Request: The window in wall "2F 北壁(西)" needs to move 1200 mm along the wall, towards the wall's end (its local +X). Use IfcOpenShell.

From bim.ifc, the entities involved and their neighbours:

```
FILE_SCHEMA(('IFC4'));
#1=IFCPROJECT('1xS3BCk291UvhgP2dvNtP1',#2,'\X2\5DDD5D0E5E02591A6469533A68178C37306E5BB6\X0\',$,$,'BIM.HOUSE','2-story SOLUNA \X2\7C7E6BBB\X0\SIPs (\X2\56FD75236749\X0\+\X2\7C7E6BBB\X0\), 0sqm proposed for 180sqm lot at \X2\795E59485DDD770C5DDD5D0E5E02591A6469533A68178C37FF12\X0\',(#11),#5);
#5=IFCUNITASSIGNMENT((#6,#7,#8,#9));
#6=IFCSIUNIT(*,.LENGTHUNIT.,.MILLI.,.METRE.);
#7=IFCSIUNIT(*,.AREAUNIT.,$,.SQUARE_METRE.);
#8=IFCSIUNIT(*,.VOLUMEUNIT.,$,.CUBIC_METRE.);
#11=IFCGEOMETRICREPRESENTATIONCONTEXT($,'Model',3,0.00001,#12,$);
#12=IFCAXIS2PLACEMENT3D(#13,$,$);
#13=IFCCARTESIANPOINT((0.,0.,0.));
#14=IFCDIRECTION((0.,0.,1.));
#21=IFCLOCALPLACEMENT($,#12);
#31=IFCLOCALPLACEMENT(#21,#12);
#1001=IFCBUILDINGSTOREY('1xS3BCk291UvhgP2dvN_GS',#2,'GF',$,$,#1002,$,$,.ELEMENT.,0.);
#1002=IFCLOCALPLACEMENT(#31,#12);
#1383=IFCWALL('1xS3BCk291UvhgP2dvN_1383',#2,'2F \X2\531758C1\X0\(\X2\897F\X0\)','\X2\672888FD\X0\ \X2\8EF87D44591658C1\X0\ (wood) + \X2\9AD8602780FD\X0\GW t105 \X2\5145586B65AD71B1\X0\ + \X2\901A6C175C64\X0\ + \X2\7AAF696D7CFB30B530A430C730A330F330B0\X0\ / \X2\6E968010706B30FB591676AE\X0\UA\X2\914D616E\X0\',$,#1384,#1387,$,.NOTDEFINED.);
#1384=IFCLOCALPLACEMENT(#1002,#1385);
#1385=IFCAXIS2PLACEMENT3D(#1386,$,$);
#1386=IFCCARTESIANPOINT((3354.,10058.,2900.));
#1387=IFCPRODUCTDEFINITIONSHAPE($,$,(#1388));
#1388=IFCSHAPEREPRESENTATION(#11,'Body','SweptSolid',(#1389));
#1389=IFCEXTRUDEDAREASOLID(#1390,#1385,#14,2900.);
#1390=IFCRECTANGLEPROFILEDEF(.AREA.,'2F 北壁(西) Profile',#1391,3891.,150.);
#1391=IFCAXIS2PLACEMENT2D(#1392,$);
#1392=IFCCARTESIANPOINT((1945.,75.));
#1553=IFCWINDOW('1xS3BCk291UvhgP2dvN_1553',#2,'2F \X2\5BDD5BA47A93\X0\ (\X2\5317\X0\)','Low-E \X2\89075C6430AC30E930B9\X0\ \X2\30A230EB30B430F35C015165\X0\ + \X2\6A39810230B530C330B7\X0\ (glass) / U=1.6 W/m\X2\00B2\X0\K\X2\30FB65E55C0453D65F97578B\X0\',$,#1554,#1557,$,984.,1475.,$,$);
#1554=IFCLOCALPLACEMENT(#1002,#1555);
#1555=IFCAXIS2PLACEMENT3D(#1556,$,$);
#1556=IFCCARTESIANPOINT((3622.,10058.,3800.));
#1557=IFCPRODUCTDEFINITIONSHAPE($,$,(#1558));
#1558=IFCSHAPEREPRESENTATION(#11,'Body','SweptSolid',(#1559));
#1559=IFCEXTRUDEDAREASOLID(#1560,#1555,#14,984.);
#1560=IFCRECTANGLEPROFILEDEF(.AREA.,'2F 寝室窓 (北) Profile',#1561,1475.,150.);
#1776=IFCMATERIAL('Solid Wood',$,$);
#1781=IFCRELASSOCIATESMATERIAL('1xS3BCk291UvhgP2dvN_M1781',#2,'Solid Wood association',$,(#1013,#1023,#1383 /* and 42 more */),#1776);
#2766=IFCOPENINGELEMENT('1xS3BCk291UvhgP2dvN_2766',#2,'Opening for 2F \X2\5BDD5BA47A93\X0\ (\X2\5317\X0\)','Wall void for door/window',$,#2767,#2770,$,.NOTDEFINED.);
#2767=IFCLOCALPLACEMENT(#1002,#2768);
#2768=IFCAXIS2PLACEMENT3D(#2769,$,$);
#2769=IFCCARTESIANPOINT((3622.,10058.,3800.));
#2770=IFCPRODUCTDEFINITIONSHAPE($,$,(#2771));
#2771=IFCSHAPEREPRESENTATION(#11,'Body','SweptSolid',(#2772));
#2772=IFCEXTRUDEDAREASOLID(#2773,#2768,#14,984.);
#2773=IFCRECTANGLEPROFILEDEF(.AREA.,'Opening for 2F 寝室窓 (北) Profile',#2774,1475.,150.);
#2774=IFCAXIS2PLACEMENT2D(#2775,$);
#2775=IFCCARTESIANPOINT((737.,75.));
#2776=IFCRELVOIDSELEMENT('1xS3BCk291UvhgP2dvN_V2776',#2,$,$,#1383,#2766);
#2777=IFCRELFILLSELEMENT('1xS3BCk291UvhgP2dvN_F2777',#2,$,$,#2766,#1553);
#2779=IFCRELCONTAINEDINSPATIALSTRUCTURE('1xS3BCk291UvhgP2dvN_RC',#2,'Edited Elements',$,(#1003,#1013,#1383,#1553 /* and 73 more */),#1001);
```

```python
import ifcopenshell
import ifcopenshell.api.geometry
import ifcopenshell.util.placement
import ifcopenshell.util.unit

model = ifcopenshell.open("bim.ifc")
unit_scale = ifcopenshell.util.unit.calculate_unit_scale(model)

window = model.by_guid("1xS3BCk291UvhgP2dvN_1553")
opening = window.FillsVoids[0].RelatingOpeningElement
wall = opening.VoidsElements[0].RelatingBuildingElement

wall_matrix = ifcopenshell.util.placement.get_local_placement(wall.ObjectPlacement)
shift = wall_matrix[:3, 0] * 1.2 / unit_scale
before = ifcopenshell.util.placement.get_local_placement(window.ObjectPlacement)[:3, 3].copy()

# The window is not placed relative to its opening, so move both.
for product in (opening, window):
    matrix = ifcopenshell.util.placement.get_local_placement(product.ObjectPlacement)
    matrix[:3, 3] += shift
    ifcopenshell.api.geometry.edit_object_placement(model, product=product, matrix=matrix, is_si=False)

after = ifcopenshell.util.placement.get_local_placement(window.ObjectPlacement)[:3, 3]
print("window moved by", (after - before).round(3) + 0.0)

model.write("bim-out.ifc")
```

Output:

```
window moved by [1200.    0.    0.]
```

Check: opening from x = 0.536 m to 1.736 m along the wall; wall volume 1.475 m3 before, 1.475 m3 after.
